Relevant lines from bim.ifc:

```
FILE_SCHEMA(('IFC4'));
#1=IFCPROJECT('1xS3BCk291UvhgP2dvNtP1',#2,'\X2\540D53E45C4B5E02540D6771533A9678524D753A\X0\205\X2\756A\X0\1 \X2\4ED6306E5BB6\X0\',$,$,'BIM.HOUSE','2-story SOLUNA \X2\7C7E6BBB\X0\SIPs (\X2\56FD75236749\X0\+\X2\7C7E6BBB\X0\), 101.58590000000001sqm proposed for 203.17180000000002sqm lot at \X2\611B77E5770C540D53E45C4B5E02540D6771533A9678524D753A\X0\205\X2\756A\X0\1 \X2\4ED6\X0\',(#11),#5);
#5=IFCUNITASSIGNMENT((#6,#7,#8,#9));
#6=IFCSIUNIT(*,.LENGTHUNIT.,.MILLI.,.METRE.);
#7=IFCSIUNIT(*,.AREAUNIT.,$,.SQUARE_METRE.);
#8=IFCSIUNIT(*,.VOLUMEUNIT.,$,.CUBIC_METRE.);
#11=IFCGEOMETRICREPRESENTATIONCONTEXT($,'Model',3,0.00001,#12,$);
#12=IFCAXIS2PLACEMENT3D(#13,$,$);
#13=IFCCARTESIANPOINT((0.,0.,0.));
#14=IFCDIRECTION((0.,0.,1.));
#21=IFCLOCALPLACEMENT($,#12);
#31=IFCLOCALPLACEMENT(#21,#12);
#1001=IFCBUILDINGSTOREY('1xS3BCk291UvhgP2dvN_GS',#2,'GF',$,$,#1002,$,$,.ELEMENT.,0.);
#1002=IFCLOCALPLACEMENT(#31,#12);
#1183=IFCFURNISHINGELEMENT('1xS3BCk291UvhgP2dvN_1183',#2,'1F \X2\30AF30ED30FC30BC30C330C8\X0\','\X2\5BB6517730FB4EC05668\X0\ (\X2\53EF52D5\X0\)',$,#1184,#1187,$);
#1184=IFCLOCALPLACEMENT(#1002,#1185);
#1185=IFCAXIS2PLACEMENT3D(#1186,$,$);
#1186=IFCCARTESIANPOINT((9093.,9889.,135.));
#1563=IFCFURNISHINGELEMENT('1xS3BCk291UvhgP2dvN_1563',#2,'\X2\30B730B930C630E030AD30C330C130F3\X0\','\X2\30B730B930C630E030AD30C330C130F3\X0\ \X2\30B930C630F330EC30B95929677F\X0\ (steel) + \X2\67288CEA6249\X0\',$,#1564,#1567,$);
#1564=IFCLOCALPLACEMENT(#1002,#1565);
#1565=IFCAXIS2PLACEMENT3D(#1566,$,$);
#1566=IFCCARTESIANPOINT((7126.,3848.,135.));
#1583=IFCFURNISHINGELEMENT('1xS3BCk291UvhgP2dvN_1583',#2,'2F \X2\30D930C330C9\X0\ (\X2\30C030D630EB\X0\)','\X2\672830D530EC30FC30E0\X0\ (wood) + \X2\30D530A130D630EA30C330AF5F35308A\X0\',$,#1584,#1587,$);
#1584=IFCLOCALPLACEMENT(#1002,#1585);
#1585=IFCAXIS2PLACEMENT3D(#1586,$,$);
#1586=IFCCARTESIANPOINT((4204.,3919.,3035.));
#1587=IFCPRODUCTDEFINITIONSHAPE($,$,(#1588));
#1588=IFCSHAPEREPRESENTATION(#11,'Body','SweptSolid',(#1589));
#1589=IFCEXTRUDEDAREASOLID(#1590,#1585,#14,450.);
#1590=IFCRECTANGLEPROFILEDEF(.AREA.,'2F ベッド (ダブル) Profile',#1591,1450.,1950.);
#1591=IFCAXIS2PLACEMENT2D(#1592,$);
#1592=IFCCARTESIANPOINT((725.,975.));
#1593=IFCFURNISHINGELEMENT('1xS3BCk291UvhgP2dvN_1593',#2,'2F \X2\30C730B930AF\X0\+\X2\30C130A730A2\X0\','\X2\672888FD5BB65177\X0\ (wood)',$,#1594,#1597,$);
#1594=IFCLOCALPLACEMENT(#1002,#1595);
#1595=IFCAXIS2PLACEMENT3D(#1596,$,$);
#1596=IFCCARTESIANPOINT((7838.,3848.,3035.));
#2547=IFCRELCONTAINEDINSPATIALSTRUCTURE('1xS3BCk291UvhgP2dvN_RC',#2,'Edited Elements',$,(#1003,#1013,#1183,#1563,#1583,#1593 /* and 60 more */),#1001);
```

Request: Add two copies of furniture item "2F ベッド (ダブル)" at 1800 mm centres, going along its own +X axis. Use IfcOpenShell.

```python
import ifcopenshell
import ifcopenshell.api.geometry
import ifcopenshell.api.root
import ifcopenshell.util.element
import ifcopenshell.util.placement
import ifcopenshell.util.unit

model = ifcopenshell.open("bim.ifc")
unit_scale = ifcopenshell.util.unit.calculate_unit_scale(model)


def reuse_history(source, copy):
    """copy_class also copies each property set's owner history, people and application; keep the originals."""
    for rel in copy.IsDefinedBy:
        if rel.is_a("IfcRelDefinesByProperties") and (history := rel.RelatingPropertyDefinition.OwnerHistory):
            rel.RelatingPropertyDefinition.OwnerHistory = source.OwnerHistory
            ifcopenshell.util.element.remove_deep2(model, history)


source = model.by_guid("1xS3BCk291UvhgP2dvN_1583")
base = ifcopenshell.util.placement.get_local_placement(source.ObjectPlacement)
step = base[:3, 0] * 1.8 / unit_scale

for i in range(1, 3):
    copy = ifcopenshell.api.root.copy_class(model, product=source)
    copy.Representation = ifcopenshell.util.element.copy_deep(
        model, source.Representation, exclude=["IfcGeometricRepresentationContext", "IfcRepresentationMap"]
    )
    reuse_history(source, copy)
    matrix = base.copy()
    matrix[:3, 3] += i * step
    print("added at", matrix[:3, 3].round(3) + 0.0)
    ifcopenshell.api.geometry.edit_object_placement(model, product=copy, matrix=matrix, is_si=False)

model.write("bim-out.ifc")
```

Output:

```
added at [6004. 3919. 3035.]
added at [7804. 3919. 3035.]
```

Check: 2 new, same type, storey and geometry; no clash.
